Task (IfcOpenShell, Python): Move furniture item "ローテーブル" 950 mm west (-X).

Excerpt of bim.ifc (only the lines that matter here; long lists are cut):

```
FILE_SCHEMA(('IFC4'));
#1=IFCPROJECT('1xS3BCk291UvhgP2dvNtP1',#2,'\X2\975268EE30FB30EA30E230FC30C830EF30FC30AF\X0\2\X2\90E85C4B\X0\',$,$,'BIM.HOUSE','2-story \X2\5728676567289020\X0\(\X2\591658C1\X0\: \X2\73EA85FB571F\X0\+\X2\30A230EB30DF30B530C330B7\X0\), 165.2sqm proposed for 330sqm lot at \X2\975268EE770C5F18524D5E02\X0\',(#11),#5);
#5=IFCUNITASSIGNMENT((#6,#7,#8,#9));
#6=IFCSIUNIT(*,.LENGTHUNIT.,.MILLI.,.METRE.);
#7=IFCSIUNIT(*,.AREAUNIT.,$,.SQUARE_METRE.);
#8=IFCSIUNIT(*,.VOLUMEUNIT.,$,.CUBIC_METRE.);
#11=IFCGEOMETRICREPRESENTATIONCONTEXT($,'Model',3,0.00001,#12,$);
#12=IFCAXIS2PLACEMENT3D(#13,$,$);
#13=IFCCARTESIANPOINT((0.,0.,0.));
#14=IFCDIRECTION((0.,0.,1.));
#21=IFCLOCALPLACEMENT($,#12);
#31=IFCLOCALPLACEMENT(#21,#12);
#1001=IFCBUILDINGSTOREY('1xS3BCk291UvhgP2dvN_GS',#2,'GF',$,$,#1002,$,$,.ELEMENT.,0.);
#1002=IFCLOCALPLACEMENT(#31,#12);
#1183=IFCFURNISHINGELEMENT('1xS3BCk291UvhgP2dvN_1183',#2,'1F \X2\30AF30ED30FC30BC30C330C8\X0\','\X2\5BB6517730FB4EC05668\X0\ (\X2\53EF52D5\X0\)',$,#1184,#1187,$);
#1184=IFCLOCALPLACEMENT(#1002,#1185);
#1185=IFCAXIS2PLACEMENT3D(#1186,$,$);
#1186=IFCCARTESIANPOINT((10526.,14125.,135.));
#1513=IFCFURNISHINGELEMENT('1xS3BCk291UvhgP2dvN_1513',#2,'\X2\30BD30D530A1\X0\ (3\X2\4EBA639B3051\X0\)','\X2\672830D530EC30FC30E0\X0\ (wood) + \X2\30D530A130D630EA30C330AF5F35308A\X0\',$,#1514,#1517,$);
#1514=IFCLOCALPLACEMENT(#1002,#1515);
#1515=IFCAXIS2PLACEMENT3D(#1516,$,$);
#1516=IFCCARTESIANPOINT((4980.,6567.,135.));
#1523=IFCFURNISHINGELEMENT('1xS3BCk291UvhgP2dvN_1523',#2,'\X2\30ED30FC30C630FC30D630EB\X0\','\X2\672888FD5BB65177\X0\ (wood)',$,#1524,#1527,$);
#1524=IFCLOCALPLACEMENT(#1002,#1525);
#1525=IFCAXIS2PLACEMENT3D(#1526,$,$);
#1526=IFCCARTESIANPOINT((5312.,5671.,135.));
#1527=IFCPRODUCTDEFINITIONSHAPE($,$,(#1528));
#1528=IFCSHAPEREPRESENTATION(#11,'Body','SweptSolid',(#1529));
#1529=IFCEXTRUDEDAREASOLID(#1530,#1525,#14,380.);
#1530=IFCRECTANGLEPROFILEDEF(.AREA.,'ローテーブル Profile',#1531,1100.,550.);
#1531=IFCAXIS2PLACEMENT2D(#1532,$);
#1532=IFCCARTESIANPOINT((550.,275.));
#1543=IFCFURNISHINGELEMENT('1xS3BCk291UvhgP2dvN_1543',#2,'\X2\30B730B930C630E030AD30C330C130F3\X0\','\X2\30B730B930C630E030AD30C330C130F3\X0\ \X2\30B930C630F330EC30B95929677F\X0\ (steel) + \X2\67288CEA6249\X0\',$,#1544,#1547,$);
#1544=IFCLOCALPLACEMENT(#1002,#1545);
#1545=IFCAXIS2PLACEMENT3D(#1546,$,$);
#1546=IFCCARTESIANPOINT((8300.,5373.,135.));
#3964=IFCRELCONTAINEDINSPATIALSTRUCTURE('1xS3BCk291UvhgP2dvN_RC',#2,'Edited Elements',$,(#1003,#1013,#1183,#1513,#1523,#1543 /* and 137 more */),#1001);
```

```python
import ifcopenshell
import ifcopenshell.api.geometry
import ifcopenshell.util.placement
import ifcopenshell.util.unit

model = ifcopenshell.open("bim.ifc")
unit_scale = ifcopenshell.util.unit.calculate_unit_scale(model)

item = model.by_id(1523)
matrix = ifcopenshell.util.placement.get_local_placement(item.ObjectPlacement)
matrix[0, 3] -= 0.95 / unit_scale
ifcopenshell.api.geometry.edit_object_placement(model, product=item, matrix=matrix, is_si=False)

print(ifcopenshell.util.placement.get_local_placement(item.ObjectPlacement).round(3) + 0.0)

model.write("bim-out.ifc")
```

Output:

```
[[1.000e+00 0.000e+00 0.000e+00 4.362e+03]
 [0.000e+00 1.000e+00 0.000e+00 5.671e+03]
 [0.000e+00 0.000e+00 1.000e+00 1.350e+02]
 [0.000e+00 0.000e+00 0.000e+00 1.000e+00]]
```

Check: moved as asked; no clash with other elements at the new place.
